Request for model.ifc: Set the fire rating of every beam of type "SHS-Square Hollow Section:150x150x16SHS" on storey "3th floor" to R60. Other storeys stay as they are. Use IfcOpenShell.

First a look at what the model holds.

```python
import ifcopenshell
import ifcopenshell.util.element

model = ifcopenshell.open("model.ifc")
print(model.schema)
storey = next(s for s in model.by_type("IfcBuildingStorey") if s.Name == "3th floor")
beams = [e for e in ifcopenshell.util.element.get_decomposition(storey) if e.is_a("IfcBeam")]
seen = {}
for e in beams:
    element_type = ifcopenshell.util.element.get_type(e)
    key = (element_type.Name if element_type != e and element_type else None, ifcopenshell.util.element.get_pset(e, "Pset_BeamCommon", "FireRating"))
    seen[key] = seen.get(key, 0) + 1
for (name, value), count in sorted(seen.items(), key=str):
    print(count, "x", name, "|", value)
```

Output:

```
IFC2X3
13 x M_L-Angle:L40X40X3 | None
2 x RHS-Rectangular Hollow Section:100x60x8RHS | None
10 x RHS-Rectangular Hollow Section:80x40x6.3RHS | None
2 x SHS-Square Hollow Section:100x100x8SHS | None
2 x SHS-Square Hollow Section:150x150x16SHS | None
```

```python
import ifcopenshell
import ifcopenshell.api.pset
import ifcopenshell.util.element

model = ifcopenshell.open("model.ifc")

storey = next(s for s in model.by_type("IfcBuildingStorey") if s.Name == "3th floor")
beams = [e for e in ifcopenshell.util.element.get_decomposition(storey) if e.is_a("IfcBeam")]

count = 0
for e in beams:
    element_type = ifcopenshell.util.element.get_type(e)
    if element_type in (None, e) or element_type.Name != "SHS-Square Hollow Section:150x150x16SHS":
        continue
    # add_pset returns the element's existing set when there is one.
    pset = ifcopenshell.api.pset.add_pset(model, product=e, name="Pset_BeamCommon")
    ifcopenshell.api.pset.edit_pset(model, pset=pset, properties={"FireRating": "R60"})
    count += 1

print(count, "beams updated")

model.write("model_edited.ifc")
```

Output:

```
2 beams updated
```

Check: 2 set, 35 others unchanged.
